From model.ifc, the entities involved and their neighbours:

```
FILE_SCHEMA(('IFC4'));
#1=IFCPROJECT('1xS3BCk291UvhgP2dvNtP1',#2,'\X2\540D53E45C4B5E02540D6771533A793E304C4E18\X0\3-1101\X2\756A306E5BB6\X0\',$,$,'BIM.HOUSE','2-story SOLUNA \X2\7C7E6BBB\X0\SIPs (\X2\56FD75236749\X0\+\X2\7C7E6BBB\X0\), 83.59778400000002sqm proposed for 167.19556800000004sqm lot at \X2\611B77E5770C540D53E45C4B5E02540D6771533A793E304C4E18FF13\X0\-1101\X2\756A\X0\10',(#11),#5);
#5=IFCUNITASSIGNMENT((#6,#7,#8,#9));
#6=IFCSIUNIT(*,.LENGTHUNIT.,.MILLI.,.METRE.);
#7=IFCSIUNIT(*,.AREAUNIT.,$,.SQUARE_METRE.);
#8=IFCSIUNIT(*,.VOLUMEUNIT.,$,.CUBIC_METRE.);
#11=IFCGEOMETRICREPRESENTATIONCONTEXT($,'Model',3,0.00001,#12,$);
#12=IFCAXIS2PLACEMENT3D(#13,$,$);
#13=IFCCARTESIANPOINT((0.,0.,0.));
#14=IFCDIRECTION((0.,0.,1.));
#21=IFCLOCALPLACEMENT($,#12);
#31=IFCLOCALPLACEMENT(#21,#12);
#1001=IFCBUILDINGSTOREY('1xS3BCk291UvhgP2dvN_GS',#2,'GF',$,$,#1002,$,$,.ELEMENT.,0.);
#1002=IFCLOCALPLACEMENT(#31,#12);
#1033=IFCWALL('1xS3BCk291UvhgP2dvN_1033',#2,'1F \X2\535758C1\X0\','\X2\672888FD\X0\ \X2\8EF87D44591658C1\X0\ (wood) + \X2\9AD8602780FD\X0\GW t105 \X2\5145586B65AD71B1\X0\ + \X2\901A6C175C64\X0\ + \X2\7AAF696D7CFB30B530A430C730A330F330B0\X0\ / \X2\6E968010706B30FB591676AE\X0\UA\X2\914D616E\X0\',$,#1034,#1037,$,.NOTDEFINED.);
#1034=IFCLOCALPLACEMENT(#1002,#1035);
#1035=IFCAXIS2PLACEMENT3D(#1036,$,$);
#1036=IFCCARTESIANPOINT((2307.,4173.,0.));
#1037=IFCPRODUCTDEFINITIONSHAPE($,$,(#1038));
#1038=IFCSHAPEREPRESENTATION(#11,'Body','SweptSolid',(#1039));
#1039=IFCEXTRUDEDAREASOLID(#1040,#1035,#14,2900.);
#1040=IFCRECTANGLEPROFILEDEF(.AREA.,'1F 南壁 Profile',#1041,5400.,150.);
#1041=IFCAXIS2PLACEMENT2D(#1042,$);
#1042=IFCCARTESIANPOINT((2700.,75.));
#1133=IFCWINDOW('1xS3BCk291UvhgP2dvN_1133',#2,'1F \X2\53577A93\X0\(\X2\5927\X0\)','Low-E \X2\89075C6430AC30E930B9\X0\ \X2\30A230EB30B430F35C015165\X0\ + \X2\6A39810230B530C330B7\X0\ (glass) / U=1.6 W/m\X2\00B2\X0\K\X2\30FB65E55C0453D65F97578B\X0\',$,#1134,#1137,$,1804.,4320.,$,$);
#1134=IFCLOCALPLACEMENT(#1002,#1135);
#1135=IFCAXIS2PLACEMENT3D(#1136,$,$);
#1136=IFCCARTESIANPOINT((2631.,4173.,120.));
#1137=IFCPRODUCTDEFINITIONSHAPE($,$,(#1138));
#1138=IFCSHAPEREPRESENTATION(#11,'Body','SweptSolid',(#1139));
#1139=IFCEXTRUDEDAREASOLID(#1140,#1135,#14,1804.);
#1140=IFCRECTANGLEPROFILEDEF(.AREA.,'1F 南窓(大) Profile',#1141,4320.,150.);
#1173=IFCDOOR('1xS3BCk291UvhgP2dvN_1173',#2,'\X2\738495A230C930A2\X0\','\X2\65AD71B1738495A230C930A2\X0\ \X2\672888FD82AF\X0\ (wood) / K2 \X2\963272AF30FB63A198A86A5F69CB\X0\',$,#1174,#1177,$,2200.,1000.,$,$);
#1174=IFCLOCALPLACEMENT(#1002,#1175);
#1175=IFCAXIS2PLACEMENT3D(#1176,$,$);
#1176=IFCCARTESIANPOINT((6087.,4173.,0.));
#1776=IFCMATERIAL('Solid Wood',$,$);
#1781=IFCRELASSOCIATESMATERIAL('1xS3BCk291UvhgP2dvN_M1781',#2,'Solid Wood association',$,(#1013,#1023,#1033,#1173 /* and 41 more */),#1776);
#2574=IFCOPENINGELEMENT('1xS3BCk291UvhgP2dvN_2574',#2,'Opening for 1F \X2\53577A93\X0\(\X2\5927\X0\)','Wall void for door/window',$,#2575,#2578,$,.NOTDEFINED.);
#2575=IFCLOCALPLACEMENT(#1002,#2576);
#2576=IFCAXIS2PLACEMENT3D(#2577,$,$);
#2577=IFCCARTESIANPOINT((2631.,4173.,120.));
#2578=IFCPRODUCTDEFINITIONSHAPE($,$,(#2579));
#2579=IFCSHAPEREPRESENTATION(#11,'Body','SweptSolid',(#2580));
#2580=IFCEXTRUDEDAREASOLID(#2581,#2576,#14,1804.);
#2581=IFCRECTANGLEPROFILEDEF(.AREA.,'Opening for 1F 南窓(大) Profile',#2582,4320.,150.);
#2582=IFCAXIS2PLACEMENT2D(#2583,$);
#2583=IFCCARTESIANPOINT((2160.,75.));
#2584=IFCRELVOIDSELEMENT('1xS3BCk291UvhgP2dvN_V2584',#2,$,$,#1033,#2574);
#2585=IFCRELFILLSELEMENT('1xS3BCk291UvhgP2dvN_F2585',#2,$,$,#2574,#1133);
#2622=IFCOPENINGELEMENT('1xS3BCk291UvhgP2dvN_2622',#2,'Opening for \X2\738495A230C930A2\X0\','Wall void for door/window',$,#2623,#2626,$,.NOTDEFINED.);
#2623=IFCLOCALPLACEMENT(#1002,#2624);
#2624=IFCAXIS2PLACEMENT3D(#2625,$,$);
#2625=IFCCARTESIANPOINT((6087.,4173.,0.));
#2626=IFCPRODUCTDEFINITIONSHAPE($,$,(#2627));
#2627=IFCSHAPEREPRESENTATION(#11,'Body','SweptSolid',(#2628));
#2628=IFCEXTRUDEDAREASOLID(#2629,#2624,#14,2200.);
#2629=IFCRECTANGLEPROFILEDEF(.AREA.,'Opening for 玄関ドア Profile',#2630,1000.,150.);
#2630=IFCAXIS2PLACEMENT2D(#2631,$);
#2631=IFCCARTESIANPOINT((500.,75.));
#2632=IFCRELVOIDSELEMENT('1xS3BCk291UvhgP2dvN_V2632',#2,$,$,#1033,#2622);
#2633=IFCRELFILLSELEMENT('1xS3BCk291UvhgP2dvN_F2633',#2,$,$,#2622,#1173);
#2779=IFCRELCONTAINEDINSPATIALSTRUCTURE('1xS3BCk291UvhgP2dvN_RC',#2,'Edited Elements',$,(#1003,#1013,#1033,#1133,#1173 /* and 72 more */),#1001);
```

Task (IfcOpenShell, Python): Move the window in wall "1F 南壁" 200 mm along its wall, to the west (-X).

```python
import ifcopenshell
import ifcopenshell.api.geometry
import ifcopenshell.util.placement
import ifcopenshell.util.unit

model = ifcopenshell.open("model.ifc")
unit_scale = ifcopenshell.util.unit.calculate_unit_scale(model)

window = model.by_id(1133)
opening = window.FillsVoids[0].RelatingOpeningElement
wall = opening.VoidsElements[0].RelatingBuildingElement

wall_matrix = ifcopenshell.util.placement.get_local_placement(wall.ObjectPlacement)
shift = wall_matrix[:3, 0] * -0.2 / unit_scale
before = ifcopenshell.util.placement.get_local_placement(window.ObjectPlacement)[:3, 3].copy()

# The window is not placed relative to its opening, so move both.
for product in (opening, window):
    matrix = ifcopenshell.util.placement.get_local_placement(product.ObjectPlacement)
    matrix[:3, 3] += shift
    ifcopenshell.api.geometry.edit_object_placement(model, product=product, matrix=matrix, is_si=False)

after = ifcopenshell.util.placement.get_local_placement(window.ObjectPlacement)[:3, 3]
print("window moved by", (after - before).round(3) + 0.0)

model.write("model_edited.ifc")
```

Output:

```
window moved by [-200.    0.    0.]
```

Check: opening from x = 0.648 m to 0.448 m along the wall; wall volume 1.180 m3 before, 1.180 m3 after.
